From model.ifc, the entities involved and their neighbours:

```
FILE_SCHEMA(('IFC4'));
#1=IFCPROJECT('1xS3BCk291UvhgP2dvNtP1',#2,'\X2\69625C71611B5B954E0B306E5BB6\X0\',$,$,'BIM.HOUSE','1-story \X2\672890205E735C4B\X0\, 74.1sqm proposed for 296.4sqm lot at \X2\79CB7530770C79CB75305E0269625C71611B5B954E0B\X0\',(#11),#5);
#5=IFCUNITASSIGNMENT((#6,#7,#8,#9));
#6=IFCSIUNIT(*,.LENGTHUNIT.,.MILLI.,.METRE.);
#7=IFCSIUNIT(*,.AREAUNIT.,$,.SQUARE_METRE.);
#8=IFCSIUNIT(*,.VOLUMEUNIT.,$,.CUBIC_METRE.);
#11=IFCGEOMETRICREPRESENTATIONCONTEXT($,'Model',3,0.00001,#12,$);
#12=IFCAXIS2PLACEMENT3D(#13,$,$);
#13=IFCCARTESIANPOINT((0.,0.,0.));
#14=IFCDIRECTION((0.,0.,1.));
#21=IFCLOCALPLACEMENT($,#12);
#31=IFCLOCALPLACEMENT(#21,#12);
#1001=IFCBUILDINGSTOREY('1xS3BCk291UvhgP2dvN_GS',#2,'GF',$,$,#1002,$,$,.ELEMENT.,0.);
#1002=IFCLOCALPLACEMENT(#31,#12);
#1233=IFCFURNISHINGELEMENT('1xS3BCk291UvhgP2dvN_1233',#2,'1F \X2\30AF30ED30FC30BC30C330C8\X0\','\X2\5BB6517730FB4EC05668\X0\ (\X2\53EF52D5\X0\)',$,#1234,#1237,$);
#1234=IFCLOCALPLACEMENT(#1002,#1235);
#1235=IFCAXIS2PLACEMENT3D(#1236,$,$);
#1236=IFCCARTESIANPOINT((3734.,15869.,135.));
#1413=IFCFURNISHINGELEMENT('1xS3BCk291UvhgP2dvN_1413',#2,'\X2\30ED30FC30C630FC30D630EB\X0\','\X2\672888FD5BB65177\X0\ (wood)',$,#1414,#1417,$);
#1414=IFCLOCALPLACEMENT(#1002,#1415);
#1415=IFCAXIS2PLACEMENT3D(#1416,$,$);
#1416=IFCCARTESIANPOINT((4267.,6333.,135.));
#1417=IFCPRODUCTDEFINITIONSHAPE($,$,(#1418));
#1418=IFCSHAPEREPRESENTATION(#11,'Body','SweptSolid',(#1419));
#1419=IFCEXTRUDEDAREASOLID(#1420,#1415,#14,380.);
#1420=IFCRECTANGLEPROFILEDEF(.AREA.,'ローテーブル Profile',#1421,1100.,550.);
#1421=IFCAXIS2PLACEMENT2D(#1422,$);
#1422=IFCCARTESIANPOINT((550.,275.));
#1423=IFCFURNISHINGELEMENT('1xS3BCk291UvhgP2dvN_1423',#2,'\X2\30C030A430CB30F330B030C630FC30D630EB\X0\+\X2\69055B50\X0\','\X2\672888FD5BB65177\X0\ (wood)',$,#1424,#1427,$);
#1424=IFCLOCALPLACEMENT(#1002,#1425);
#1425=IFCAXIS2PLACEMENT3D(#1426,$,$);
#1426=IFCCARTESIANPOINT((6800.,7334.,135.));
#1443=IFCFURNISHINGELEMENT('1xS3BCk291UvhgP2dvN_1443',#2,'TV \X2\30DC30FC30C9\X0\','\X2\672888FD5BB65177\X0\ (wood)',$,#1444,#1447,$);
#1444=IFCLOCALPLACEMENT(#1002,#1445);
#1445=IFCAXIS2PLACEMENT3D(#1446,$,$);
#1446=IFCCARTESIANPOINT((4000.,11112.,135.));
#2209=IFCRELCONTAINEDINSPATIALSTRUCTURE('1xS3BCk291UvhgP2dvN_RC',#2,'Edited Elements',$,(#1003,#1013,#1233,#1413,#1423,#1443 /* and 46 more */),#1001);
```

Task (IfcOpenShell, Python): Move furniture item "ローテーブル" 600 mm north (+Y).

```python
import ifcopenshell
import ifcopenshell.api.geometry
import ifcopenshell.util.placement

model = ifcopenshell.open("model.ifc")

item = model.by_guid("1xS3BCk291UvhgP2dvN_1413")
matrix = ifcopenshell.util.placement.get_local_placement(item.ObjectPlacement)
matrix[1, 3] += 600.0
ifcopenshell.api.geometry.edit_object_placement(model, product=item, matrix=matrix, is_si=False)

print(ifcopenshell.util.placement.get_local_placement(item.ObjectPlacement).round(3) + 0.0)

model.write("model-out.ifc")
```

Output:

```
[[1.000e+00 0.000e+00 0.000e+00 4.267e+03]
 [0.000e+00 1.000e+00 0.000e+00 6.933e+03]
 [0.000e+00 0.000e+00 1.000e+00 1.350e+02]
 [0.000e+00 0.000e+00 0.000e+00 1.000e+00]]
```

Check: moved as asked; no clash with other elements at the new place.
